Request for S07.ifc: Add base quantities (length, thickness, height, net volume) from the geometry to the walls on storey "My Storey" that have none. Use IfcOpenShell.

First a look at what the model holds.

```python
import ifcopenshell
import ifcopenshell.util.element
import ifcopenshell.util.unit

model = ifcopenshell.open("S07.ifc")
print(model.schema)
for unit_type in ("LENGTHUNIT", "AREAUNIT", "VOLUMEUNIT"):
    print(unit_type, ifcopenshell.util.unit.calculate_unit_scale(model, unit_type))
storey = next(s for s in model.by_type("IfcBuildingStorey") if s.Name == "My Storey")
walls = [e for e in ifcopenshell.util.element.get_decomposition(storey) if e.is_a("IfcWall")]
for e in sorted(walls, key=lambda e: e.id()):
    print(e.id(), e.is_a(), e.Name, list(ifcopenshell.util.element.get_psets(e, qtos_only=True)), sep=" | ")
```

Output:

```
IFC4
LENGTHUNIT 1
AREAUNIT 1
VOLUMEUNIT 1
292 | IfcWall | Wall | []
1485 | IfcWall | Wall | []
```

```python
import ifcopenshell
import ifcopenshell.api.pset
import ifcopenshell.geom
import ifcopenshell.util.element
import ifcopenshell.util.shape
import ifcopenshell.util.unit

model = ifcopenshell.open("S07.ifc")
unit_scale = ifcopenshell.util.unit.calculate_unit_scale(model)
volume_scale = ifcopenshell.util.unit.calculate_unit_scale(model, "VOLUMEUNIT")
settings = ifcopenshell.geom.settings()

storey = next(s for s in model.by_type("IfcBuildingStorey") if s.Name == "My Storey")
walls = [e for e in ifcopenshell.util.element.get_decomposition(storey) if e.is_a("IfcWall")]

for e in sorted(walls, key=lambda e: e.id()):
    if ifcopenshell.util.element.get_psets(e, qtos_only=True, should_inherit=False):
        continue
    # Geometry comes back in metres, in the element's own axes.
    shape = ifcopenshell.geom.create_shape(settings, e)
    values = {
        "Length": ifcopenshell.util.shape.get_x(shape.geometry) / unit_scale,
        "Width": ifcopenshell.util.shape.get_y(shape.geometry) / unit_scale,
        "Height": ifcopenshell.util.shape.get_z(shape.geometry) / unit_scale,
        "NetVolume": ifcopenshell.util.shape.get_volume(shape.geometry) / volume_scale,
    }
    qto = ifcopenshell.api.pset.add_qto(model, product=e, name="Qto_WallBaseQuantities")
    ifcopenshell.api.pset.edit_qto(model, qto=qto, properties=values)
    print(e.id(), {k: round(v, 3) for k, v in values.items()})

model.write("S07_rev.ifc")
```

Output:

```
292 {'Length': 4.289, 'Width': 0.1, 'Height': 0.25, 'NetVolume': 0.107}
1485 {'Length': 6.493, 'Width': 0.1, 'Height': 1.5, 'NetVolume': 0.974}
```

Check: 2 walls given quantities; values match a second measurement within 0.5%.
